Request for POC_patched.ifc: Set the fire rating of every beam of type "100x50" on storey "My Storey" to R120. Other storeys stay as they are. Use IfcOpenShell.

First a look at what the model holds.

```python
import ifcopenshell
import ifcopenshell.util.element

model = ifcopenshell.open("POC_patched.ifc")
print(model.schema)
storey = next(s for s in model.by_type("IfcBuildingStorey") if s.Name == "My Storey")
beams = [e for e in ifcopenshell.util.element.get_decomposition(storey) if e.is_a("IfcBeam")]
seen = {}
for e in beams:
    element_type = ifcopenshell.util.element.get_type(e)
    key = (element_type.Name if element_type != e and element_type else None, ifcopenshell.util.element.get_pset(e, "Pset_BeamCommon", "FireRating"))
    seen[key] = seen.get(key, 0) + 1
for (name, value), count in sorted(seen.items(), key=str):
    print(count, "x", name, "|", value)
```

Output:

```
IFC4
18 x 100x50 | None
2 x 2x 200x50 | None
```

```python
import ifcopenshell
import ifcopenshell.api.pset
import ifcopenshell.util.element

model = ifcopenshell.open("POC_patched.ifc")

storey = next(s for s in model.by_type("IfcBuildingStorey") if s.Name == "My Storey")
beams = [e for e in ifcopenshell.util.element.get_decomposition(storey) if e.is_a("IfcBeam")]

count = 0
for e in beams:
    element_type = ifcopenshell.util.element.get_type(e)
    if element_type in (None, e) or element_type.Name != "100x50":
        continue
    # add_pset returns the element's existing set when there is one.
    pset = ifcopenshell.api.pset.add_pset(model, product=e, name="Pset_BeamCommon")
    ifcopenshell.api.pset.edit_pset(model, pset=pset, properties={"FireRating": "R120"})
    count += 1

print(count, "beams updated")

model.write("POC_patched_updated.ifc")
```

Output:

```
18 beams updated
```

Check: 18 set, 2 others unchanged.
